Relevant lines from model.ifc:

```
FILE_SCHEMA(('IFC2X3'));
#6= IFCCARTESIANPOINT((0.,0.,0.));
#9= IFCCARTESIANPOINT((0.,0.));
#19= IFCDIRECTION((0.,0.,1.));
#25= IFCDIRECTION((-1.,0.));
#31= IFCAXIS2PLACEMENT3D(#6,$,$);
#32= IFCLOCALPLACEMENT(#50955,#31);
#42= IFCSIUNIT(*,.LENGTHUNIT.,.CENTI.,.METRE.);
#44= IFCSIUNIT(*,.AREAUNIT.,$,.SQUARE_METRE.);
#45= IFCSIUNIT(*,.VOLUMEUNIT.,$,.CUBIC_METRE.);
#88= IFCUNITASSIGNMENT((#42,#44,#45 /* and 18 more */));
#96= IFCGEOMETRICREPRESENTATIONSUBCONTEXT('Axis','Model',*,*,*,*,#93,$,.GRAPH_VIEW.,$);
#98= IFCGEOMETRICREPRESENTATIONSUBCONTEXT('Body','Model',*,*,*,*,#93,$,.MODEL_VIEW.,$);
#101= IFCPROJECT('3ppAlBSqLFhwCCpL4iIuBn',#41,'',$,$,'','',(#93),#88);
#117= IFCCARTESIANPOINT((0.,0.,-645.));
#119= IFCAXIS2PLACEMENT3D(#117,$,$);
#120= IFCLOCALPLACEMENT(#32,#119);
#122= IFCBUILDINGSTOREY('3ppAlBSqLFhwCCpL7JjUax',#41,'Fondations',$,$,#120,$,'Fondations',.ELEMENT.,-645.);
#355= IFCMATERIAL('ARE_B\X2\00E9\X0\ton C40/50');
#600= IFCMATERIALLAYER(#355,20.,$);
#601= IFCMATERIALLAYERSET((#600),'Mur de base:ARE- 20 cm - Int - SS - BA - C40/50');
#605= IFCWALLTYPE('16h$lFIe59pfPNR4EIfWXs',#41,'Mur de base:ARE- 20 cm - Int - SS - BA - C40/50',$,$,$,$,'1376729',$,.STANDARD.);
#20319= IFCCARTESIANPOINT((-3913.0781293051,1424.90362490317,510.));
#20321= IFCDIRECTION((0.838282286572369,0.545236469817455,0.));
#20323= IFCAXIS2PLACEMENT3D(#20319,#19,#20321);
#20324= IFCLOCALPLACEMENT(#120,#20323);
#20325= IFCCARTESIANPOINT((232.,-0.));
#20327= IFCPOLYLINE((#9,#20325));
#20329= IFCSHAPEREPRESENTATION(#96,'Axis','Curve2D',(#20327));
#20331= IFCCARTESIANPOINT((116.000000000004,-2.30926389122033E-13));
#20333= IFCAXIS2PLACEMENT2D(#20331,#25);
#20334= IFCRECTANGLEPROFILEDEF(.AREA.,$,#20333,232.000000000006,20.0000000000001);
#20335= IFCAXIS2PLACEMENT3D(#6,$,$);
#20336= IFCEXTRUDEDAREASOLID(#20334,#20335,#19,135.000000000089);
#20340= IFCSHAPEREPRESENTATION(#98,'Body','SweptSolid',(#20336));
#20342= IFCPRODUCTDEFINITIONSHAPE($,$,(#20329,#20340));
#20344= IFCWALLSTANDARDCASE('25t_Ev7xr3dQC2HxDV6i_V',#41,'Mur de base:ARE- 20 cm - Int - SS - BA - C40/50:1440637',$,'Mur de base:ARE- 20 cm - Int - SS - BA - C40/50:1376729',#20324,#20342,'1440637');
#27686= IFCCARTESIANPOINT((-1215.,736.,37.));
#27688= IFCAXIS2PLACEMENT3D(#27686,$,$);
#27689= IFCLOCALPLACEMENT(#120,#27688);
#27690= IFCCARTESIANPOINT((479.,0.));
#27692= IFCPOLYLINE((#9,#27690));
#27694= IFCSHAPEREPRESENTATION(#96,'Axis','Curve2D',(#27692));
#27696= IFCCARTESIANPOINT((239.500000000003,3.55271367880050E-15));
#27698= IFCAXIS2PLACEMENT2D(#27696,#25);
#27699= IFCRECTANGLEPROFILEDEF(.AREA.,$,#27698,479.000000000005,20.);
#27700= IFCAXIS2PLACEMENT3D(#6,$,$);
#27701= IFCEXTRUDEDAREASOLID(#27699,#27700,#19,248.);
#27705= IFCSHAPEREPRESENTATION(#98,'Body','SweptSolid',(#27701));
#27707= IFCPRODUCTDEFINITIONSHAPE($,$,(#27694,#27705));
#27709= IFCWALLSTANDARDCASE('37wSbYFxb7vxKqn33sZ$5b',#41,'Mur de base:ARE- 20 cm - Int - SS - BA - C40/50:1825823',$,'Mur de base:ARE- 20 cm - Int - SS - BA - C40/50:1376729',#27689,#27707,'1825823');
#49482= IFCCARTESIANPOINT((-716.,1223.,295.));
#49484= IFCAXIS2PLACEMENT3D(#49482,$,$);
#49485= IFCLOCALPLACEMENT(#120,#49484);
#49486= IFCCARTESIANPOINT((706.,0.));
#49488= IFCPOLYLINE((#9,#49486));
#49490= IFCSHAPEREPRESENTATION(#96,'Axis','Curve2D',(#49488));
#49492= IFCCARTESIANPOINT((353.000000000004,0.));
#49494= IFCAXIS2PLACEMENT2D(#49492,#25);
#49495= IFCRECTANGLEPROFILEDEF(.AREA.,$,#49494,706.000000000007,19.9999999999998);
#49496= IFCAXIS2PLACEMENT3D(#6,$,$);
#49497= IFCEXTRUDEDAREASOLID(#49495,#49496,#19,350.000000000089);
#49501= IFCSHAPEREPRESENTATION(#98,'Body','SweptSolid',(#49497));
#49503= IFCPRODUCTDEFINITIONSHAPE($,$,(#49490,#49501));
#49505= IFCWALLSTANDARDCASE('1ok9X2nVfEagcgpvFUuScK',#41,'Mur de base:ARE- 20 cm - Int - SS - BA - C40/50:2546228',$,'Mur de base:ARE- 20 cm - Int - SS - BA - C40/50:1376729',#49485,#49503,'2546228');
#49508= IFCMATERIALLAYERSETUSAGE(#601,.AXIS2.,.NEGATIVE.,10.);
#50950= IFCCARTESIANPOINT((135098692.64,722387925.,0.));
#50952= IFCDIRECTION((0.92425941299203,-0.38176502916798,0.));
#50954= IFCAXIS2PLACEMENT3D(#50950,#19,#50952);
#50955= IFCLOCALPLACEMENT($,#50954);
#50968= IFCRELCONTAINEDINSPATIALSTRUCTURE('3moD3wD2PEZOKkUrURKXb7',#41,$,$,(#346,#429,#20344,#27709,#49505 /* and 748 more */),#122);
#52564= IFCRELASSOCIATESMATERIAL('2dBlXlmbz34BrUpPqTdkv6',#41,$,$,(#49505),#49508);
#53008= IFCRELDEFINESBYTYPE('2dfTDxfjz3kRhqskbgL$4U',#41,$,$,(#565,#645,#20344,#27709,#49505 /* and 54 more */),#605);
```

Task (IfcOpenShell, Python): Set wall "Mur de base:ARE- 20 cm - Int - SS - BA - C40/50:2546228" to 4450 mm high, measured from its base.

```python
import ifcopenshell
import ifcopenshell.geom
import ifcopenshell.util.representation
import ifcopenshell.util.shape
import ifcopenshell.util.unit

model = ifcopenshell.open("model.ifc")
unit_scale = ifcopenshell.util.unit.calculate_unit_scale(model)
settings = ifcopenshell.geom.settings()


def volume(element):
    """Net volume in cubic metres, openings subtracted."""
    shape = ifcopenshell.geom.create_shape(settings, element)
    return ifcopenshell.util.shape.get_volume(shape.geometry)


wall = model.by_id(49505)
before = volume(wall)

body = ifcopenshell.util.representation.get_representation(wall, "Model", "Body")
solid = body.Items[0]
old_height = solid.Depth
solid.Depth = 4.45 / unit_scale
after = volume(wall)

print(f"height {old_height:g} -> {solid.Depth:g}, volume {before:.3f} -> {after:.3f} m3")

model.write("model_edited.ifc")
```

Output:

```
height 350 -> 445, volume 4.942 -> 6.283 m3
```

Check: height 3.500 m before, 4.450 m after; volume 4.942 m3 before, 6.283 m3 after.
